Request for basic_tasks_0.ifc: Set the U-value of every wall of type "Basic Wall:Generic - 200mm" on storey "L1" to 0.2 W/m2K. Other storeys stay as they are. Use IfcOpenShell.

First a look at what the model holds.

```python
import ifcopenshell
import ifcopenshell.util.element

model = ifcopenshell.open("basic_tasks_0.ifc")
print(model.schema)
storey = next(s for s in model.by_type("IfcBuildingStorey") if s.Name == "L1")
walls = [e for e in ifcopenshell.util.element.get_decomposition(storey) if e.is_a("IfcWall")]
seen = {}
for e in walls:
    element_type = ifcopenshell.util.element.get_type(e)
    key = (element_type.Name if element_type != e and element_type else None, ifcopenshell.util.element.get_pset(e, "Pset_WallCommon", "ThermalTransmittance"))
    seen[key] = seen.get(key, 0) + 1
for (name, value), count in sorted(seen.items(), key=str):
    print(count, "x", name, "|", value)
```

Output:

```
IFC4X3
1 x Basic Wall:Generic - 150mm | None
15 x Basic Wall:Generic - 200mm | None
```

```python
import ifcopenshell
import ifcopenshell.api.pset
import ifcopenshell.util.element

model = ifcopenshell.open("basic_tasks_0.ifc")

storey = next(s for s in model.by_type("IfcBuildingStorey") if s.Name == "L1")
walls = [e for e in ifcopenshell.util.element.get_decomposition(storey) if e.is_a("IfcWall")]

count = 0
for e in walls:
    element_type = ifcopenshell.util.element.get_type(e)
    if element_type in (None, e) or element_type.Name != "Basic Wall:Generic - 200mm":
        continue
    # add_pset returns the element's existing set when there is one.
    pset = ifcopenshell.api.pset.add_pset(model, product=e, name="Pset_WallCommon")
    ifcopenshell.api.pset.edit_pset(model, pset=pset, properties={"ThermalTransmittance": 0.2})
    count += 1

print(count, "walls updated")

model.write("basic_tasks_0_rev.ifc")
```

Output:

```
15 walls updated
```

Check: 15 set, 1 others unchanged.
